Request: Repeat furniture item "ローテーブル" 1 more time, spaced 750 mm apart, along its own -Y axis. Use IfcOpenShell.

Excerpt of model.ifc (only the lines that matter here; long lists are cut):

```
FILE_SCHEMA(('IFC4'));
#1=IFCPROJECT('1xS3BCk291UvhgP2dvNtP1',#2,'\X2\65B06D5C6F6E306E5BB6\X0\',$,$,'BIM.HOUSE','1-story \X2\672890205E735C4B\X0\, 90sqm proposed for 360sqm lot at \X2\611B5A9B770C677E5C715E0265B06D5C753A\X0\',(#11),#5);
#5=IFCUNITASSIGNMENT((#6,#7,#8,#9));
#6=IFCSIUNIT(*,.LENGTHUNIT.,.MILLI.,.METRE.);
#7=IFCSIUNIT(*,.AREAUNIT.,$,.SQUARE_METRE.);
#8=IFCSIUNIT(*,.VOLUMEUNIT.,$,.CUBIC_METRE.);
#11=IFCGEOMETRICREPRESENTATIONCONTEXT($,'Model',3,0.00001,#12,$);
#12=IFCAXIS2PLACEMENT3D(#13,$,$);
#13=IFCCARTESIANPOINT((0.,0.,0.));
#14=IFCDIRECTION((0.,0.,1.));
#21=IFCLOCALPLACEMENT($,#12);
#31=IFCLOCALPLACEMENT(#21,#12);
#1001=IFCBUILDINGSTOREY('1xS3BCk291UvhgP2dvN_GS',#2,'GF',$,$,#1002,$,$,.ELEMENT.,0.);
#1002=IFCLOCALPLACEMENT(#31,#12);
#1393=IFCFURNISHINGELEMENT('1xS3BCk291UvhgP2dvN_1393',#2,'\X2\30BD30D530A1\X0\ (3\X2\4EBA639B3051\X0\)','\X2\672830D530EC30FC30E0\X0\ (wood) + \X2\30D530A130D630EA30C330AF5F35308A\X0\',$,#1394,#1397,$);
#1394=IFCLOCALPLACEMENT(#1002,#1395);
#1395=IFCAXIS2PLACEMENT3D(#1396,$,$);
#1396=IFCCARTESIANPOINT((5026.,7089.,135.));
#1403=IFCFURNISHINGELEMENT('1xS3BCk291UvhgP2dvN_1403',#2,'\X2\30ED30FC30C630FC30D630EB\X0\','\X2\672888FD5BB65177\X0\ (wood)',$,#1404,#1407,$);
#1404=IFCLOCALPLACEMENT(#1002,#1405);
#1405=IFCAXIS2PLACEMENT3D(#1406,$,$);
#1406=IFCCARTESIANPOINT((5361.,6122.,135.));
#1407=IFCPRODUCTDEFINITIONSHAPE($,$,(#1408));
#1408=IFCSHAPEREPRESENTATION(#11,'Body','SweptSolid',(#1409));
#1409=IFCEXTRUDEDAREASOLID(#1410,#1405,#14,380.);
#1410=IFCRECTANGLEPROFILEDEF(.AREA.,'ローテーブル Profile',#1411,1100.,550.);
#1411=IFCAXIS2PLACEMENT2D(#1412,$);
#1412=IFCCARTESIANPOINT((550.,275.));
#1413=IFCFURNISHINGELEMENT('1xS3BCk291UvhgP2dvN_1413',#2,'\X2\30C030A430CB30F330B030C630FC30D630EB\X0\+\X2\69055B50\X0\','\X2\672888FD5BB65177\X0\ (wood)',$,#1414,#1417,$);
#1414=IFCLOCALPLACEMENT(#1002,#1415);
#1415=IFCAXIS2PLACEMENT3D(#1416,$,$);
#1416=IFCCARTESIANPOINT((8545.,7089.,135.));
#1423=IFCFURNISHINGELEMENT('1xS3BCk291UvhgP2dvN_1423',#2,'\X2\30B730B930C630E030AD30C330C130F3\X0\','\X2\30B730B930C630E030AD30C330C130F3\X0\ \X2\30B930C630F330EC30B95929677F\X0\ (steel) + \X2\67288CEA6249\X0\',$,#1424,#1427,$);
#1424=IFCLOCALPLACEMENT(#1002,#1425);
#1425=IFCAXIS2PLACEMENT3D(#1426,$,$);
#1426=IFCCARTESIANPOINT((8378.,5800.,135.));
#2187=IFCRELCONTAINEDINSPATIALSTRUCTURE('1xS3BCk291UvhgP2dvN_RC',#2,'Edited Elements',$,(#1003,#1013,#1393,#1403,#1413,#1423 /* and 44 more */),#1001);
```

```python
import ifcopenshell
import ifcopenshell.api.geometry
import ifcopenshell.api.root
import ifcopenshell.util.element
import ifcopenshell.util.placement

model = ifcopenshell.open("model.ifc")


def reuse_history(source, copy):
    """copy_class also copies each property set's owner history, people and application; keep the originals."""
    for rel in copy.IsDefinedBy:
        if rel.is_a("IfcRelDefinesByProperties") and (history := rel.RelatingPropertyDefinition.OwnerHistory):
            rel.RelatingPropertyDefinition.OwnerHistory = source.OwnerHistory
            ifcopenshell.util.element.remove_deep2(model, history)


source = model.by_guid("1xS3BCk291UvhgP2dvN_1403")
base = ifcopenshell.util.placement.get_local_placement(source.ObjectPlacement)
step = -base[:3, 1] * 750.0

for i in range(1, 2):
    copy = ifcopenshell.api.root.copy_class(model, product=source)
    copy.Representation = ifcopenshell.util.element.copy_deep(
        model, source.Representation, exclude=["IfcGeometricRepresentationContext", "IfcRepresentationMap"]
    )
    reuse_history(source, copy)
    matrix = base.copy()
    matrix[:3, 3] += i * step
    print("added at", matrix[:3, 3].round(3) + 0.0)
    ifcopenshell.api.geometry.edit_object_placement(model, product=copy, matrix=matrix, is_si=False)

model.write("model_v2.ifc")
```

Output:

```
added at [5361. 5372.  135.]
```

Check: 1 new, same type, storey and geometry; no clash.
